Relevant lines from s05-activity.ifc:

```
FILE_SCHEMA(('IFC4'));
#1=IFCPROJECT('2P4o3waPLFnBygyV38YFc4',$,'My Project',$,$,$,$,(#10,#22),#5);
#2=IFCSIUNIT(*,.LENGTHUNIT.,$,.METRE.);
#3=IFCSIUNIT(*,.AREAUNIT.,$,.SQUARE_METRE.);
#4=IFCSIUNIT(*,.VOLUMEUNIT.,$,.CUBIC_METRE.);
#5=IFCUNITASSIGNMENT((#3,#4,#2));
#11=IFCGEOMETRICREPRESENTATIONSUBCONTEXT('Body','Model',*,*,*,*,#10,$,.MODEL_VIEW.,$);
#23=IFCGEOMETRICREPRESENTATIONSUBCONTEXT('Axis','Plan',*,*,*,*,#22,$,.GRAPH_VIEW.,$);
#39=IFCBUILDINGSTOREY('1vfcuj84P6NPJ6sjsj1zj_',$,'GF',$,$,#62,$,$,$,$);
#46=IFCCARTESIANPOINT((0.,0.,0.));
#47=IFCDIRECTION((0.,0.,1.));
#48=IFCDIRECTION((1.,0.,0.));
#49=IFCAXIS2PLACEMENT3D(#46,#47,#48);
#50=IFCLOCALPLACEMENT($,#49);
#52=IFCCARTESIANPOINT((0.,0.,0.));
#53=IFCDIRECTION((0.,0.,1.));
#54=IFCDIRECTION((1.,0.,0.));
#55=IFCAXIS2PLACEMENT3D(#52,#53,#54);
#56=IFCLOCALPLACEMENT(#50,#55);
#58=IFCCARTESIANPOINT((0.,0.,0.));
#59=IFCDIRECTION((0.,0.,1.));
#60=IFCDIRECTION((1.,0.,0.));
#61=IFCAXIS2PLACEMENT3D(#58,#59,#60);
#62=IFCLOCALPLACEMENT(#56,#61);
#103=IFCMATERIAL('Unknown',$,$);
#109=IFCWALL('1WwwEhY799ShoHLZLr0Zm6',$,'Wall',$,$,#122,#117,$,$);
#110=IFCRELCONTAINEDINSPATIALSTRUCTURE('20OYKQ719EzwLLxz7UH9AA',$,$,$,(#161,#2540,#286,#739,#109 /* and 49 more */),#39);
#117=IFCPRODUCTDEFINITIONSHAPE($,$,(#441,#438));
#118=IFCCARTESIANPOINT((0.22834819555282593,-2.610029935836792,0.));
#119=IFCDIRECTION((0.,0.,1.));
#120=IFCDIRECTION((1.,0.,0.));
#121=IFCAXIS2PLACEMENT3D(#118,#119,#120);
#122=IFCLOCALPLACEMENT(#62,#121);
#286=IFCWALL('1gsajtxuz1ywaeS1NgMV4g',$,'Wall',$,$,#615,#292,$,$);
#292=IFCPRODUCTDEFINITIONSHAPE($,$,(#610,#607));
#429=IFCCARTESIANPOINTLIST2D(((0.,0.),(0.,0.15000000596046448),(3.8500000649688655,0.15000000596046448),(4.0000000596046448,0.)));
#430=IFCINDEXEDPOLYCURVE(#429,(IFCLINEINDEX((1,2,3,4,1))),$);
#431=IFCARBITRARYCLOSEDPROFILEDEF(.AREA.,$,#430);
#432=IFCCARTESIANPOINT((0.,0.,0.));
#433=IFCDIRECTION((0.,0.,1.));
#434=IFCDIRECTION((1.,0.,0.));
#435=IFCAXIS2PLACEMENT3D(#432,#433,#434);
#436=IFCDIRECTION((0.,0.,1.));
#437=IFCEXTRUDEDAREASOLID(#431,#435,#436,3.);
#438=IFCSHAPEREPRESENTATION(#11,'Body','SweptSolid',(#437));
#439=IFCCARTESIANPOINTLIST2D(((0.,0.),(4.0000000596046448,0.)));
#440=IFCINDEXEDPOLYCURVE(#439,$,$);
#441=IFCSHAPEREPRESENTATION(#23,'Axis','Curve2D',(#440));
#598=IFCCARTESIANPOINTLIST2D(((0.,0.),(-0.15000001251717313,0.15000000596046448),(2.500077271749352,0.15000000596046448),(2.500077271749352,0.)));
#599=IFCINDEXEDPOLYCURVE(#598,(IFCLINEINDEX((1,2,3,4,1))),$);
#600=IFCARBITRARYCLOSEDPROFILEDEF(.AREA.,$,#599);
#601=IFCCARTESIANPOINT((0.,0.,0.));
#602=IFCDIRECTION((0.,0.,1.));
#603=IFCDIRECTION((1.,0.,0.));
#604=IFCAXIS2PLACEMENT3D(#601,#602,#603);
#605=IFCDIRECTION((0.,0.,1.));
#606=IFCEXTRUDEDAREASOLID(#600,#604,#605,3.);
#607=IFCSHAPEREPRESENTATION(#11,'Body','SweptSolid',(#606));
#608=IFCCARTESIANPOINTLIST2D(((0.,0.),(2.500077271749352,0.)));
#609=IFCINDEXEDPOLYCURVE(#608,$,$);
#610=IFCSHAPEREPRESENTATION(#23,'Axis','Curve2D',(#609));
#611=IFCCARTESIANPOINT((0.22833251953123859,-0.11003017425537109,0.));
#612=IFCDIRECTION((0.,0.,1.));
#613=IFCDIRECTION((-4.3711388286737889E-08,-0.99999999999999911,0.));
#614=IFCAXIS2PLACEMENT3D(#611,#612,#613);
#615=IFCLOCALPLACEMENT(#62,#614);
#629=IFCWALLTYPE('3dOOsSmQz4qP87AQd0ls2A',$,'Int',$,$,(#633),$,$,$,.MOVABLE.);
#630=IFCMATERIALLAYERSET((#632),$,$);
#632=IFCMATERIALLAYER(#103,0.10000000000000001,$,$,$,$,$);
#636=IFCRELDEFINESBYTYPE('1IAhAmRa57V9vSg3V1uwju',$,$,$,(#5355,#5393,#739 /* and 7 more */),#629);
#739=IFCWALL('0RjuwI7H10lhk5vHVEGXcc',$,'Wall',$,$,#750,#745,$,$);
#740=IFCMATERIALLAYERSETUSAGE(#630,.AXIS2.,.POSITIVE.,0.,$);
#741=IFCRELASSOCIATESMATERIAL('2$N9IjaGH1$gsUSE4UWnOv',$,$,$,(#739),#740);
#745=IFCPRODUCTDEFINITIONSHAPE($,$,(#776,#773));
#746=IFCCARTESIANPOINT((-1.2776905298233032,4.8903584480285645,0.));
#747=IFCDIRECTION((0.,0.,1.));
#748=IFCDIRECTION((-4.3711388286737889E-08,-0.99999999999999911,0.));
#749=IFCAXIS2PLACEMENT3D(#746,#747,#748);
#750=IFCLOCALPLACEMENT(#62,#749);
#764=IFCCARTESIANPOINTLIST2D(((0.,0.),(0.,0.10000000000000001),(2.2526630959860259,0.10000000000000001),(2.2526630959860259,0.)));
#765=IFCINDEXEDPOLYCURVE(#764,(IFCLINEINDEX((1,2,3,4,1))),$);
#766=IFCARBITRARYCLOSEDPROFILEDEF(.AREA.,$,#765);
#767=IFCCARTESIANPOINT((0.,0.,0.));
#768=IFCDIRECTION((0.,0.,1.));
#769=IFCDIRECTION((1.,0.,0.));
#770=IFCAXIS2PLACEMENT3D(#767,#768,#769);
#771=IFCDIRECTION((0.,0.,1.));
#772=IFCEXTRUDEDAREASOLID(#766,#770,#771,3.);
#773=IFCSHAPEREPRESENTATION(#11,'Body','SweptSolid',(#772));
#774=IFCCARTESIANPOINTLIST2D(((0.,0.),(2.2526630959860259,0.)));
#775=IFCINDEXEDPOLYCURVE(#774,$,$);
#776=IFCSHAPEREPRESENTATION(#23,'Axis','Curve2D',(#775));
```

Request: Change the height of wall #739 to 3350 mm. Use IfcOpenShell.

```python
import ifcopenshell
import ifcopenshell.geom
import ifcopenshell.util.representation
import ifcopenshell.util.shape
import ifcopenshell.util.unit

model = ifcopenshell.open("s05-activity.ifc")
unit_scale = ifcopenshell.util.unit.calculate_unit_scale(model)
settings = ifcopenshell.geom.settings()


def volume(element):
    """Net volume in cubic metres, openings subtracted."""
    shape = ifcopenshell.geom.create_shape(settings, element)
    return ifcopenshell.util.shape.get_volume(shape.geometry)


wall = model.by_id(739)
before = volume(wall)

body = ifcopenshell.util.representation.get_representation(wall, "Model", "Body")
solid = body.Items[0]
old_height = solid.Depth
solid.Depth = 3.35 / unit_scale
after = volume(wall)

print(f"height {old_height:g} -> {solid.Depth:g}, volume {before:.3f} -> {after:.3f} m3")

model.write("s05-activity_edited.ifc")
```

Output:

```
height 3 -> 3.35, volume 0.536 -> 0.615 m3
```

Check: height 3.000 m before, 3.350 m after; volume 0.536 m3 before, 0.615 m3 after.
